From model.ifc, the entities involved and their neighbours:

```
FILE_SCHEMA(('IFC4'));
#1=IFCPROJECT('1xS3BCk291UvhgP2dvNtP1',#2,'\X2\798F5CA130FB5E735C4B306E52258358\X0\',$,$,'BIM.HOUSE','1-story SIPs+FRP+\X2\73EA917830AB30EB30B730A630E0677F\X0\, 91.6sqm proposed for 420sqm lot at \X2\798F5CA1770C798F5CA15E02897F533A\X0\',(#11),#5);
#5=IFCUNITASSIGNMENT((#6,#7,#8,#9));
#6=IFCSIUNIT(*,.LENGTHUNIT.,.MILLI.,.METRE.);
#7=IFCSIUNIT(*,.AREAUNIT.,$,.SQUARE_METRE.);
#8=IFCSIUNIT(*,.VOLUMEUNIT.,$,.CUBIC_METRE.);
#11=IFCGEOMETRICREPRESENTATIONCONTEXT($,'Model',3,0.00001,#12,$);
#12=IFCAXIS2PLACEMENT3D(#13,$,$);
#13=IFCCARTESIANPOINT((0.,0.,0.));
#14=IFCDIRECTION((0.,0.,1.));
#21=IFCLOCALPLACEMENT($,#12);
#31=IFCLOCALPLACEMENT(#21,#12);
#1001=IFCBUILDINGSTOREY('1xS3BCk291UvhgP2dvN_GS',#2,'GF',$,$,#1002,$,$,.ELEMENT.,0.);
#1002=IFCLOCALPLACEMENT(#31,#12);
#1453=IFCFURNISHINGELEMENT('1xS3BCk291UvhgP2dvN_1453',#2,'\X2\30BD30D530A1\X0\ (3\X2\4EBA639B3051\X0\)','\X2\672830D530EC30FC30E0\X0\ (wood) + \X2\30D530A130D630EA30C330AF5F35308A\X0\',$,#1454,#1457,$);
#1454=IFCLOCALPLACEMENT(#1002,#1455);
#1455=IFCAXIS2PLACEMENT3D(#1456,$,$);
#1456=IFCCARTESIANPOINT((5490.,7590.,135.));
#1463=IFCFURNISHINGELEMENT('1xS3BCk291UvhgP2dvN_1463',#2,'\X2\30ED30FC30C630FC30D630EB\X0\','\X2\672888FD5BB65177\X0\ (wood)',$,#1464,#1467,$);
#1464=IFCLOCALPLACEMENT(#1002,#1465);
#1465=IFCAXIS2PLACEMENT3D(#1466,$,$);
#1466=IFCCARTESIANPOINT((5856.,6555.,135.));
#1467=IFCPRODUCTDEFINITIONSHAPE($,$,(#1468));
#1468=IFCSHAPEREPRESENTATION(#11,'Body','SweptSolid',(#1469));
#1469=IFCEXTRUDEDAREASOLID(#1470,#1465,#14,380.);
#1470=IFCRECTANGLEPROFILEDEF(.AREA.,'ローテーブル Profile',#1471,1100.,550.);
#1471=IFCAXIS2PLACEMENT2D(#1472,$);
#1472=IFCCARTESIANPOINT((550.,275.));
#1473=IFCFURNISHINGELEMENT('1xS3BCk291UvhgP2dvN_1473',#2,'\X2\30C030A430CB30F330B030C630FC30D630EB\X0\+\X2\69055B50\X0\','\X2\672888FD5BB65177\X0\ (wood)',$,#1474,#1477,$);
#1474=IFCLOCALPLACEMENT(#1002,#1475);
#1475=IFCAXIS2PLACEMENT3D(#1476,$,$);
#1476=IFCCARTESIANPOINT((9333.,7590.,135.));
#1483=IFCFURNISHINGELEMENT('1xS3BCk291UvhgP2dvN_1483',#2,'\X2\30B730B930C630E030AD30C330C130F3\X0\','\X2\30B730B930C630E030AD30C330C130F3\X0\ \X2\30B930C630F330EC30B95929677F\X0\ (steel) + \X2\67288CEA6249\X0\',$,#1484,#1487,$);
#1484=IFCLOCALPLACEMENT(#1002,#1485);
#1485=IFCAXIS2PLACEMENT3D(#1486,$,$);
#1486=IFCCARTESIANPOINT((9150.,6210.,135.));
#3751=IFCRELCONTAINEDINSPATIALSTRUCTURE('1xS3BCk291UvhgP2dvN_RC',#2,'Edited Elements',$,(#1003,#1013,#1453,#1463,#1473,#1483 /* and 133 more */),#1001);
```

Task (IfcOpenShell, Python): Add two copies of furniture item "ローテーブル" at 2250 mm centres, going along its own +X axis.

```python
import ifcopenshell
import ifcopenshell.api.geometry
import ifcopenshell.api.root
import ifcopenshell.util.element
import ifcopenshell.util.placement
import ifcopenshell.util.unit

model = ifcopenshell.open("model.ifc")
unit_scale = ifcopenshell.util.unit.calculate_unit_scale(model)


def reuse_history(source, copy):
    """copy_class also copies each property set's owner history, people and application; keep the originals."""
    for rel in copy.IsDefinedBy:
        if rel.is_a("IfcRelDefinesByProperties") and (history := rel.RelatingPropertyDefinition.OwnerHistory):
            rel.RelatingPropertyDefinition.OwnerHistory = source.OwnerHistory
            ifcopenshell.util.element.remove_deep2(model, history)


source = model.by_guid("1xS3BCk291UvhgP2dvN_1463")
base = ifcopenshell.util.placement.get_local_placement(source.ObjectPlacement)
step = base[:3, 0] * 2.25 / unit_scale

for i in range(1, 3):
    copy = ifcopenshell.api.root.copy_class(model, product=source)
    copy.Representation = ifcopenshell.util.element.copy_deep(
        model, source.Representation, exclude=["IfcGeometricRepresentationContext", "IfcRepresentationMap"]
    )
    reuse_history(source, copy)
    matrix = base.copy()
    matrix[:3, 3] += i * step
    print("added at", matrix[:3, 3].round(3) + 0.0)
    ifcopenshell.api.geometry.edit_object_placement(model, product=copy, matrix=matrix, is_si=False)

model.write("model-out.ifc")
```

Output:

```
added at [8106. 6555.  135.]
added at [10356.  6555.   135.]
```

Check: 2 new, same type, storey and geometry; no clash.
